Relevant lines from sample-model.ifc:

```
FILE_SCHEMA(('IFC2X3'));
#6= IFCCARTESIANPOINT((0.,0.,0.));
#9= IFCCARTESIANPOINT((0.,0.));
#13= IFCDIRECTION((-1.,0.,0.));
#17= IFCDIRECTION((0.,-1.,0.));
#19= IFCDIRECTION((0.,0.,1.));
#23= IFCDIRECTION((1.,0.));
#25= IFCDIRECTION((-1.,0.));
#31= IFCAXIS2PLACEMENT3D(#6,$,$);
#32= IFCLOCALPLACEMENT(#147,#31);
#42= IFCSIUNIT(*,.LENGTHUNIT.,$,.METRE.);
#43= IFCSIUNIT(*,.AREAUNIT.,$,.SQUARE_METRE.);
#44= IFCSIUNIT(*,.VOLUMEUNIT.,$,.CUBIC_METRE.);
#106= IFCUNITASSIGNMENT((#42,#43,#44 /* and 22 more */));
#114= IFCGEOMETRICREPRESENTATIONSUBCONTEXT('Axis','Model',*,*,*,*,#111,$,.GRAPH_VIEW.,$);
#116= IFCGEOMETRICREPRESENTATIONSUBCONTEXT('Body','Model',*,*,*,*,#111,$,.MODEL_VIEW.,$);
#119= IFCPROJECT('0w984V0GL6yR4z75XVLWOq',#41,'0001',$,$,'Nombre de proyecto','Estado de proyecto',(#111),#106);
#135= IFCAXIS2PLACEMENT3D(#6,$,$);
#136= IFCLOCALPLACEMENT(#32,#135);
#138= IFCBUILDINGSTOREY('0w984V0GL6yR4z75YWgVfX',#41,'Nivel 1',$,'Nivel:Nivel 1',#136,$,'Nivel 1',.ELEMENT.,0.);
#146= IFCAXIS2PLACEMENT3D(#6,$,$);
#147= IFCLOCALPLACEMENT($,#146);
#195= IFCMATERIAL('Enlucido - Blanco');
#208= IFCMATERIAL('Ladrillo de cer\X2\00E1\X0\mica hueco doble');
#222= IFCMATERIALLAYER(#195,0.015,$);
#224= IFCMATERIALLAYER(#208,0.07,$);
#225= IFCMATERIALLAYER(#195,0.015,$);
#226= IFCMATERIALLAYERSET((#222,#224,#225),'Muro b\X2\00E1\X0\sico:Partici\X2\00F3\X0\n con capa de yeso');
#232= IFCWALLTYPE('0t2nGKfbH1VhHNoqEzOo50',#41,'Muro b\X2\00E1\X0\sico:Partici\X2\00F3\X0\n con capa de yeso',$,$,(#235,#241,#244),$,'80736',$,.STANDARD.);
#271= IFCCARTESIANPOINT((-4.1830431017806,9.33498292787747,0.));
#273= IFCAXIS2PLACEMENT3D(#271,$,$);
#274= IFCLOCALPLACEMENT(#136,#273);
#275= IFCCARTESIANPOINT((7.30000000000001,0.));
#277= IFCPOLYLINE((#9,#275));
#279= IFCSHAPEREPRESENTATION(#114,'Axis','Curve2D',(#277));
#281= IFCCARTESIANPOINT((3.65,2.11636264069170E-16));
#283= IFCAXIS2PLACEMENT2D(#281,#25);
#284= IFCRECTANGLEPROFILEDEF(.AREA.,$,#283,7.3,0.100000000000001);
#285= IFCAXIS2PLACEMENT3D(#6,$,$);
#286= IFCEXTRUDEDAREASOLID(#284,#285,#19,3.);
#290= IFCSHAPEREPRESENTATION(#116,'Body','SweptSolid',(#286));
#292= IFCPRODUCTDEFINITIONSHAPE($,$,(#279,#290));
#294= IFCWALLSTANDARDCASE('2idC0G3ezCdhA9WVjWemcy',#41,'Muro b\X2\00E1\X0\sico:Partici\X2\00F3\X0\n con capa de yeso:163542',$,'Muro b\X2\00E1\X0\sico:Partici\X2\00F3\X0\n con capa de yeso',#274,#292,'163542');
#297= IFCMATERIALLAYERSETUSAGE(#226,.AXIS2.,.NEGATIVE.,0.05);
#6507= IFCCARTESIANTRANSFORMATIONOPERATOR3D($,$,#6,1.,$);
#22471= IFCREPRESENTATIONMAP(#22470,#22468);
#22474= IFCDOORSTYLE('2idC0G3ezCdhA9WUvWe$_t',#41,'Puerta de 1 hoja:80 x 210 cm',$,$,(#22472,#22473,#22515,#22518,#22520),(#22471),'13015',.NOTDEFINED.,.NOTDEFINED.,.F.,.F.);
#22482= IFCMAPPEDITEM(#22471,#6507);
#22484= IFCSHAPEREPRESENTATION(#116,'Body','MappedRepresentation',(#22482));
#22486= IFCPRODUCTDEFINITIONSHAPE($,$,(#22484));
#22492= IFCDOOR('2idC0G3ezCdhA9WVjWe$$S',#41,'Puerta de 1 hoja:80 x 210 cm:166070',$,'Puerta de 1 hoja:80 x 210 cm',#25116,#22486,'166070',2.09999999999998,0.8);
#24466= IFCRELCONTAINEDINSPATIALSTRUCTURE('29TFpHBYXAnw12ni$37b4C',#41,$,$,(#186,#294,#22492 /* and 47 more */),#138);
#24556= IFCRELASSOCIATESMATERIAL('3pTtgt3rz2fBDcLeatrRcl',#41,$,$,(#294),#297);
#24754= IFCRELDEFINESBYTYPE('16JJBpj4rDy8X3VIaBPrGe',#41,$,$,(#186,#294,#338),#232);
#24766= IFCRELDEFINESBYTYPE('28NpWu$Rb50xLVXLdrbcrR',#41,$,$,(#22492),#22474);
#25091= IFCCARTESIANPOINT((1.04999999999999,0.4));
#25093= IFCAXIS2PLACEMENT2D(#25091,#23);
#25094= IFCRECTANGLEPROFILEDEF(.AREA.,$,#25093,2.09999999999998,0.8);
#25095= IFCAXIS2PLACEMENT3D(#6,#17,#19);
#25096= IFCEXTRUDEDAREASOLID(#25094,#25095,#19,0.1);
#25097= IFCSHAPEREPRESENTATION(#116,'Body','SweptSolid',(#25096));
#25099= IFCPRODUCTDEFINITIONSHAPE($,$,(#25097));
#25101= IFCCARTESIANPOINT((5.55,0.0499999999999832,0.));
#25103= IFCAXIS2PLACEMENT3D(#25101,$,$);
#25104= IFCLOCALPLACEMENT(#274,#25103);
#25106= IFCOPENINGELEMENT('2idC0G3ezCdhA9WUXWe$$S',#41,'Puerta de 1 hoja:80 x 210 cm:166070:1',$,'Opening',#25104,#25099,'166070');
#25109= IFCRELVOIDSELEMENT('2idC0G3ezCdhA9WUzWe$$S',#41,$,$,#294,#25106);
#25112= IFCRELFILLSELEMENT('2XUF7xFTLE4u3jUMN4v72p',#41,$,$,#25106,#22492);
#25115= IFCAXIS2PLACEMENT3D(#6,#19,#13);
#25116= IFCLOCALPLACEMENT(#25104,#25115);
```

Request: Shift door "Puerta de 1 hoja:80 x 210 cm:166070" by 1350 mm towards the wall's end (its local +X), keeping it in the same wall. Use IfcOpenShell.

```python
import ifcopenshell
import ifcopenshell.api.geometry
import ifcopenshell.util.placement
import ifcopenshell.util.unit

model = ifcopenshell.open("sample-model.ifc")
unit_scale = ifcopenshell.util.unit.calculate_unit_scale(model)

door = model.by_guid("2idC0G3ezCdhA9WVjWe$$S")
opening = door.FillsVoids[0].RelatingOpeningElement
wall = opening.VoidsElements[0].RelatingBuildingElement

wall_matrix = ifcopenshell.util.placement.get_local_placement(wall.ObjectPlacement)
shift = wall_matrix[:3, 0] * 1.35 / unit_scale
before = ifcopenshell.util.placement.get_local_placement(door.ObjectPlacement)[:3, 3].copy()

# The door is placed relative to its opening, so it follows when the opening moves.
matrix = ifcopenshell.util.placement.get_local_placement(opening.ObjectPlacement)
matrix[:3, 3] += shift
ifcopenshell.api.geometry.edit_object_placement(
    model, product=opening, matrix=matrix, is_si=False, should_transform_children=True
)

after = ifcopenshell.util.placement.get_local_placement(door.ObjectPlacement)[:3, 3]
print("door moved by", (after - before).round(3) + 0.0)

model.write("sample-model_rev.ifc")
```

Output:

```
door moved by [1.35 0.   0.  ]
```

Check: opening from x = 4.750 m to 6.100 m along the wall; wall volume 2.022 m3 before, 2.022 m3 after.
